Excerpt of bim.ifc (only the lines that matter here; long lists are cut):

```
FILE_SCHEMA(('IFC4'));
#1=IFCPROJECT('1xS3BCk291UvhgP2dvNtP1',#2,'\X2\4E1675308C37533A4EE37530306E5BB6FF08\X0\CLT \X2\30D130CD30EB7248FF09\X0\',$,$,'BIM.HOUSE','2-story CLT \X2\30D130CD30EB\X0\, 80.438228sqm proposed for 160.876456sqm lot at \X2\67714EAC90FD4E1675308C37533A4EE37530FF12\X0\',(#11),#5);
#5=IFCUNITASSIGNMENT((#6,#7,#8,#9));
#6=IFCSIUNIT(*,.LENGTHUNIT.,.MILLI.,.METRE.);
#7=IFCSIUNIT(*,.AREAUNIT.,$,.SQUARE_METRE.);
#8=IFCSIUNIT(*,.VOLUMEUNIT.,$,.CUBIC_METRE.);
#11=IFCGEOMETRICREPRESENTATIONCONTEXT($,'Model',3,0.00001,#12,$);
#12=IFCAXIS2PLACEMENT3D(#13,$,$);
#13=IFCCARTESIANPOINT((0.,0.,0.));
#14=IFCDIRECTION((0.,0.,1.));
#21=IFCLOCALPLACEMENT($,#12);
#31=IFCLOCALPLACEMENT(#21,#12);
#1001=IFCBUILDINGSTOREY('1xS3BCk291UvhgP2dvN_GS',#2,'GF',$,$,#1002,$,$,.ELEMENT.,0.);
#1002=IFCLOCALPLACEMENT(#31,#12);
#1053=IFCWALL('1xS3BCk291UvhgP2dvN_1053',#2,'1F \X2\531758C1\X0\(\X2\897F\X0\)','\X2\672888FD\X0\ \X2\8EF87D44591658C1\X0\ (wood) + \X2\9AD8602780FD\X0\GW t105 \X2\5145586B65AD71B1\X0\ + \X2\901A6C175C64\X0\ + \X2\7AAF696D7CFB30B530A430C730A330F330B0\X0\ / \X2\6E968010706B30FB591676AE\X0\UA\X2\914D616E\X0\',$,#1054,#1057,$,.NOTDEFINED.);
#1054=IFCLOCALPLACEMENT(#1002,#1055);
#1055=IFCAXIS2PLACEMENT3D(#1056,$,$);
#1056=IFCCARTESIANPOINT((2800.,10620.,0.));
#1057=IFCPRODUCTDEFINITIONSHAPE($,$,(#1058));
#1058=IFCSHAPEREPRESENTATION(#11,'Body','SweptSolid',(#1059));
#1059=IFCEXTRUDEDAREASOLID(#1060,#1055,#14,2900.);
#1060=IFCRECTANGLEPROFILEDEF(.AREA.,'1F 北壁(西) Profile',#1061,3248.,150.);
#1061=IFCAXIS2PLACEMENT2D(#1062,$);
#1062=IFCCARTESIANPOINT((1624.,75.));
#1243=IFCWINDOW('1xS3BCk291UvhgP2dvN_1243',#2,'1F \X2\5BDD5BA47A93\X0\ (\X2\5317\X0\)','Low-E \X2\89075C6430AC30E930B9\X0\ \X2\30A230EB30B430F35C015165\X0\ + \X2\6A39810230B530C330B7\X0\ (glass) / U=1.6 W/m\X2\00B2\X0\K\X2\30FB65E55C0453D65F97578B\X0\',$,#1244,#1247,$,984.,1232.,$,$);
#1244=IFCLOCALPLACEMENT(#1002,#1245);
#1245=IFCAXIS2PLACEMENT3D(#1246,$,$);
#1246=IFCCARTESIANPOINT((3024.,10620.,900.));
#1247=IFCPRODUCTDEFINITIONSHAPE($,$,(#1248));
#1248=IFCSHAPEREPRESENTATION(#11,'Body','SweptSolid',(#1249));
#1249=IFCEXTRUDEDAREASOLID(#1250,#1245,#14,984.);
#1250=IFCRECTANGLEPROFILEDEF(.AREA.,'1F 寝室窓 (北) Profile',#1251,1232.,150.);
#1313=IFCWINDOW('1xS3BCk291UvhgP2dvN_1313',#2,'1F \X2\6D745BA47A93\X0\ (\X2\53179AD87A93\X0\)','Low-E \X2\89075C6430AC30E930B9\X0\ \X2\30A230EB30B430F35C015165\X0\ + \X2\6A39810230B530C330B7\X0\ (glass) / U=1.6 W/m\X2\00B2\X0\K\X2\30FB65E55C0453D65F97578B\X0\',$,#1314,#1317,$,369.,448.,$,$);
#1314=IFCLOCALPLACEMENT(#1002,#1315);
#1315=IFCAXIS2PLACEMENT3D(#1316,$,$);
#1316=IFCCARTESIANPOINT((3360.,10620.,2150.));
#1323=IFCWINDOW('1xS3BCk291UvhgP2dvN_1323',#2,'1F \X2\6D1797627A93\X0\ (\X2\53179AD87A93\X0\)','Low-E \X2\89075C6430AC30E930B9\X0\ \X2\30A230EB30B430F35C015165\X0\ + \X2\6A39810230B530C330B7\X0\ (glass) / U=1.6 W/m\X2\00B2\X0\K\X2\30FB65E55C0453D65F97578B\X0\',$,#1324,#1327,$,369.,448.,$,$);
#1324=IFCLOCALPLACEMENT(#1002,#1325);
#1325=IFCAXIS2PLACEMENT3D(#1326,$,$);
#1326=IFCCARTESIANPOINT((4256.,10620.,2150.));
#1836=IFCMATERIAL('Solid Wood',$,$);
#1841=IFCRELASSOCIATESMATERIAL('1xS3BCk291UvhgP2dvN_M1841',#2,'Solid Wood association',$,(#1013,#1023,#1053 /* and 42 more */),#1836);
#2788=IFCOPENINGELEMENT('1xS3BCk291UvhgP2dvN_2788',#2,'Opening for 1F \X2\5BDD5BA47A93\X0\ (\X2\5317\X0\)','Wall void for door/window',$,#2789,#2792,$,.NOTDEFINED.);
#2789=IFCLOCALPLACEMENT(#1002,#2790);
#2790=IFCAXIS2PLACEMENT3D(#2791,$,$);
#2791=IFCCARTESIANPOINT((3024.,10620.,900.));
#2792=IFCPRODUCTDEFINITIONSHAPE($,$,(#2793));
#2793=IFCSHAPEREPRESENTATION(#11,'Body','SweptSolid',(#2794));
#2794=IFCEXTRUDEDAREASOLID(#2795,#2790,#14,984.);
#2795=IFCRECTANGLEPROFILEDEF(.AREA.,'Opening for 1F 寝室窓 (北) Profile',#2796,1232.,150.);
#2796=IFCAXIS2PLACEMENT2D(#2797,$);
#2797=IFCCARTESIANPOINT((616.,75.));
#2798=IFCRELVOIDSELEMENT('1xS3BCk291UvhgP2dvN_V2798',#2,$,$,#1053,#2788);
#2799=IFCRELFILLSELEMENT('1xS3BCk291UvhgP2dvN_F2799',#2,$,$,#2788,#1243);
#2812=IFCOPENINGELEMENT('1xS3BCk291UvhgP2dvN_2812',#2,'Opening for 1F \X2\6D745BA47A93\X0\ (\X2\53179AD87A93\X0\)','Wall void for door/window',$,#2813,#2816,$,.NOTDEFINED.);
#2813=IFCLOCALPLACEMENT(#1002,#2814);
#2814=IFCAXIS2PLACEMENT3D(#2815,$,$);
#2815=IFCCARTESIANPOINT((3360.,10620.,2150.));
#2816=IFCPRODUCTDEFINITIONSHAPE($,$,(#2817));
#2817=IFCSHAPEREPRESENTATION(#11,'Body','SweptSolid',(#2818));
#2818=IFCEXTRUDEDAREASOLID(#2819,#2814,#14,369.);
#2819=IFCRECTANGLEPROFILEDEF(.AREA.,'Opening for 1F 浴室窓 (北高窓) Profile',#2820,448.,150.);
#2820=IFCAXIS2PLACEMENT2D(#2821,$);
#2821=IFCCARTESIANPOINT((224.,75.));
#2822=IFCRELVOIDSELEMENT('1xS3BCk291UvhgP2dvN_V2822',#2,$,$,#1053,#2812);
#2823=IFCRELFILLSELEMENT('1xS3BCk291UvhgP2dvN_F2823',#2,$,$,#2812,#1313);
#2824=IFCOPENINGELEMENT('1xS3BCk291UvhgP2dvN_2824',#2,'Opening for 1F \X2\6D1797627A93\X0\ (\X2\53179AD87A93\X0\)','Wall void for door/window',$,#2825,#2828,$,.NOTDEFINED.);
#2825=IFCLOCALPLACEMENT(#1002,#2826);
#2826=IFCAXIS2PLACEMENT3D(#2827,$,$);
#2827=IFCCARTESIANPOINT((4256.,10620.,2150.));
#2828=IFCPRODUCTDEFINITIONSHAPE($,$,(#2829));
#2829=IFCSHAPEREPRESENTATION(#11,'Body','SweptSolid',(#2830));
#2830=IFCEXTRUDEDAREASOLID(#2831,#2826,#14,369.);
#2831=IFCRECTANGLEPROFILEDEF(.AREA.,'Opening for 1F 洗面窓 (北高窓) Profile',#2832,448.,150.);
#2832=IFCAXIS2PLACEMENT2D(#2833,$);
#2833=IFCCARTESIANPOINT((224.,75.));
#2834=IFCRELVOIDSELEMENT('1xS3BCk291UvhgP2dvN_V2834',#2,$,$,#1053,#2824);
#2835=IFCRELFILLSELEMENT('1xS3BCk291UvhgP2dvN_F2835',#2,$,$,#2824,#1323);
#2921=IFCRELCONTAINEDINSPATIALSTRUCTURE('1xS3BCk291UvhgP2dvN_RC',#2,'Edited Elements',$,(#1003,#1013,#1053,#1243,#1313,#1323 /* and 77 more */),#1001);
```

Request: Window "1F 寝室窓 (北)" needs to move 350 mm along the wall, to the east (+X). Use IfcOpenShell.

```python
import ifcopenshell
import ifcopenshell.api.geometry
import ifcopenshell.util.placement
import ifcopenshell.util.unit

model = ifcopenshell.open("bim.ifc")
unit_scale = ifcopenshell.util.unit.calculate_unit_scale(model)

window = model.by_guid("1xS3BCk291UvhgP2dvN_1243")
opening = window.FillsVoids[0].RelatingOpeningElement
wall = opening.VoidsElements[0].RelatingBuildingElement

wall_matrix = ifcopenshell.util.placement.get_local_placement(wall.ObjectPlacement)
shift = wall_matrix[:3, 0] * 0.35 / unit_scale
before = ifcopenshell.util.placement.get_local_placement(window.ObjectPlacement)[:3, 3].copy()

# The window is not placed relative to its opening, so move both.
for product in (opening, window):
    matrix = ifcopenshell.util.placement.get_local_placement(product.ObjectPlacement)
    matrix[:3, 3] += shift
    ifcopenshell.api.geometry.edit_object_placement(model, product=product, matrix=matrix, is_si=False)

after = ifcopenshell.util.placement.get_local_placement(window.ObjectPlacement)[:3, 3]
print("window moved by", (after - before).round(3) + 0.0)

model.write("bim_v2.ifc")
```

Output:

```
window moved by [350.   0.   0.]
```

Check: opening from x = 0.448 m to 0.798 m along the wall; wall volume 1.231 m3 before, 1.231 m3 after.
